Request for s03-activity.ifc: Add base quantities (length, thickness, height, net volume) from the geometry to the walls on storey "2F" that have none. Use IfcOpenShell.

First a look at what the model holds.

```python
import ifcopenshell
import ifcopenshell.util.element
import ifcopenshell.util.unit

model = ifcopenshell.open("s03-activity.ifc")
print(model.schema)
for unit_type in ("LENGTHUNIT", "AREAUNIT", "VOLUMEUNIT"):
    print(unit_type, ifcopenshell.util.unit.calculate_unit_scale(model, unit_type))
storey = next(s for s in model.by_type("IfcBuildingStorey") if s.Name == "2F")
walls = [e for e in ifcopenshell.util.element.get_decomposition(storey) if e.is_a("IfcWall")]
for e in sorted(walls, key=lambda e: e.id()):
    print(e.id(), e.is_a(), e.Name, list(ifcopenshell.util.element.get_psets(e, qtos_only=True)), sep=" | ")
```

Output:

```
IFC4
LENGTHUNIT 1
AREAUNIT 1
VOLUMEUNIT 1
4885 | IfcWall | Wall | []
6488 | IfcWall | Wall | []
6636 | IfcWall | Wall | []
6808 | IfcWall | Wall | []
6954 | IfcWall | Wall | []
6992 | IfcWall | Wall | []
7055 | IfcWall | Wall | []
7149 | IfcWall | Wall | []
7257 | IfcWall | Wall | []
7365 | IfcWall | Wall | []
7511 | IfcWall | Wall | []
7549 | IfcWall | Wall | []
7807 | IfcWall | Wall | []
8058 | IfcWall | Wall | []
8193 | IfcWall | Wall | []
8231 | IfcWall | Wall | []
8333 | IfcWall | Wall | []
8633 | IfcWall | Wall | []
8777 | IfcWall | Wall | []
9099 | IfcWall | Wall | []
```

```python
import ifcopenshell
import ifcopenshell.api.pset
import ifcopenshell.geom
import ifcopenshell.util.element
import ifcopenshell.util.shape
import ifcopenshell.util.unit

model = ifcopenshell.open("s03-activity.ifc")
unit_scale = ifcopenshell.util.unit.calculate_unit_scale(model)
volume_scale = ifcopenshell.util.unit.calculate_unit_scale(model, "VOLUMEUNIT")
settings = ifcopenshell.geom.settings()

storey = next(s for s in model.by_type("IfcBuildingStorey") if s.Name == "2F")
walls = [e for e in ifcopenshell.util.element.get_decomposition(storey) if e.is_a("IfcWall")]

for e in sorted(walls, key=lambda e: e.id()):
    if ifcopenshell.util.element.get_psets(e, qtos_only=True, should_inherit=False):
        continue
    # Geometry comes back in metres, in the element's own axes.
    shape = ifcopenshell.geom.create_shape(settings, e)
    values = {
        "Length": ifcopenshell.util.shape.get_x(shape.geometry) / unit_scale,
        "Width": ifcopenshell.util.shape.get_y(shape.geometry) / unit_scale,
        "Height": ifcopenshell.util.shape.get_z(shape.geometry) / unit_scale,
        "NetVolume": ifcopenshell.util.shape.get_volume(shape.geometry) / volume_scale,
    }
    qto = ifcopenshell.api.pset.add_qto(model, product=e, name="Qto_WallBaseQuantities")
    ifcopenshell.api.pset.edit_qto(model, qto=qto, properties=values)
    print(e.id(), {k: round(v, 3) for k, v in values.items()})

model.write("s03-activity_edited.ifc")
```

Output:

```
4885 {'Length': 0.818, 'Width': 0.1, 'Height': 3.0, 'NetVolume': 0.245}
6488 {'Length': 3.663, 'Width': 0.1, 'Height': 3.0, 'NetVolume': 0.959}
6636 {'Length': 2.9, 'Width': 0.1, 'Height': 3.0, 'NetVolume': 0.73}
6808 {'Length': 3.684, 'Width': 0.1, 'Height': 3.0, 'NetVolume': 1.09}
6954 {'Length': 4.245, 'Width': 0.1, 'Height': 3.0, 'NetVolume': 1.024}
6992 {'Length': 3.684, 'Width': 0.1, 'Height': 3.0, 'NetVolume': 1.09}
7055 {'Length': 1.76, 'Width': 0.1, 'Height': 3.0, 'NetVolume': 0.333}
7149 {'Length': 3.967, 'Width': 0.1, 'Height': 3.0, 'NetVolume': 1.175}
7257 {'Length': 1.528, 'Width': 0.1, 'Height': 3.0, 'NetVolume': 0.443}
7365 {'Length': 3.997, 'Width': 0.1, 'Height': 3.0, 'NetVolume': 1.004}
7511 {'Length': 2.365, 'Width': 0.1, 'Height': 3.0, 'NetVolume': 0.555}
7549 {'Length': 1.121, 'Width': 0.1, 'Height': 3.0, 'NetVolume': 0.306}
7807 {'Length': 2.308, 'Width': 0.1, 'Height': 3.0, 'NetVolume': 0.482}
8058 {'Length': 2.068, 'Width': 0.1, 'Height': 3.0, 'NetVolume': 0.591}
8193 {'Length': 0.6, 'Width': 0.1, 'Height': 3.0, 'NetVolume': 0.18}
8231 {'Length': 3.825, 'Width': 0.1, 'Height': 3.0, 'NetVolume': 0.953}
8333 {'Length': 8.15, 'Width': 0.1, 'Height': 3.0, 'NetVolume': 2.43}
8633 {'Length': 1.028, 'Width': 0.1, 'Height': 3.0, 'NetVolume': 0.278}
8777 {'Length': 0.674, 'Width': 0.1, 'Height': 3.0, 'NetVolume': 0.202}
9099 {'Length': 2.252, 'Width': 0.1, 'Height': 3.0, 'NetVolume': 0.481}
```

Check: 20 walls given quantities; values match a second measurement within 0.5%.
